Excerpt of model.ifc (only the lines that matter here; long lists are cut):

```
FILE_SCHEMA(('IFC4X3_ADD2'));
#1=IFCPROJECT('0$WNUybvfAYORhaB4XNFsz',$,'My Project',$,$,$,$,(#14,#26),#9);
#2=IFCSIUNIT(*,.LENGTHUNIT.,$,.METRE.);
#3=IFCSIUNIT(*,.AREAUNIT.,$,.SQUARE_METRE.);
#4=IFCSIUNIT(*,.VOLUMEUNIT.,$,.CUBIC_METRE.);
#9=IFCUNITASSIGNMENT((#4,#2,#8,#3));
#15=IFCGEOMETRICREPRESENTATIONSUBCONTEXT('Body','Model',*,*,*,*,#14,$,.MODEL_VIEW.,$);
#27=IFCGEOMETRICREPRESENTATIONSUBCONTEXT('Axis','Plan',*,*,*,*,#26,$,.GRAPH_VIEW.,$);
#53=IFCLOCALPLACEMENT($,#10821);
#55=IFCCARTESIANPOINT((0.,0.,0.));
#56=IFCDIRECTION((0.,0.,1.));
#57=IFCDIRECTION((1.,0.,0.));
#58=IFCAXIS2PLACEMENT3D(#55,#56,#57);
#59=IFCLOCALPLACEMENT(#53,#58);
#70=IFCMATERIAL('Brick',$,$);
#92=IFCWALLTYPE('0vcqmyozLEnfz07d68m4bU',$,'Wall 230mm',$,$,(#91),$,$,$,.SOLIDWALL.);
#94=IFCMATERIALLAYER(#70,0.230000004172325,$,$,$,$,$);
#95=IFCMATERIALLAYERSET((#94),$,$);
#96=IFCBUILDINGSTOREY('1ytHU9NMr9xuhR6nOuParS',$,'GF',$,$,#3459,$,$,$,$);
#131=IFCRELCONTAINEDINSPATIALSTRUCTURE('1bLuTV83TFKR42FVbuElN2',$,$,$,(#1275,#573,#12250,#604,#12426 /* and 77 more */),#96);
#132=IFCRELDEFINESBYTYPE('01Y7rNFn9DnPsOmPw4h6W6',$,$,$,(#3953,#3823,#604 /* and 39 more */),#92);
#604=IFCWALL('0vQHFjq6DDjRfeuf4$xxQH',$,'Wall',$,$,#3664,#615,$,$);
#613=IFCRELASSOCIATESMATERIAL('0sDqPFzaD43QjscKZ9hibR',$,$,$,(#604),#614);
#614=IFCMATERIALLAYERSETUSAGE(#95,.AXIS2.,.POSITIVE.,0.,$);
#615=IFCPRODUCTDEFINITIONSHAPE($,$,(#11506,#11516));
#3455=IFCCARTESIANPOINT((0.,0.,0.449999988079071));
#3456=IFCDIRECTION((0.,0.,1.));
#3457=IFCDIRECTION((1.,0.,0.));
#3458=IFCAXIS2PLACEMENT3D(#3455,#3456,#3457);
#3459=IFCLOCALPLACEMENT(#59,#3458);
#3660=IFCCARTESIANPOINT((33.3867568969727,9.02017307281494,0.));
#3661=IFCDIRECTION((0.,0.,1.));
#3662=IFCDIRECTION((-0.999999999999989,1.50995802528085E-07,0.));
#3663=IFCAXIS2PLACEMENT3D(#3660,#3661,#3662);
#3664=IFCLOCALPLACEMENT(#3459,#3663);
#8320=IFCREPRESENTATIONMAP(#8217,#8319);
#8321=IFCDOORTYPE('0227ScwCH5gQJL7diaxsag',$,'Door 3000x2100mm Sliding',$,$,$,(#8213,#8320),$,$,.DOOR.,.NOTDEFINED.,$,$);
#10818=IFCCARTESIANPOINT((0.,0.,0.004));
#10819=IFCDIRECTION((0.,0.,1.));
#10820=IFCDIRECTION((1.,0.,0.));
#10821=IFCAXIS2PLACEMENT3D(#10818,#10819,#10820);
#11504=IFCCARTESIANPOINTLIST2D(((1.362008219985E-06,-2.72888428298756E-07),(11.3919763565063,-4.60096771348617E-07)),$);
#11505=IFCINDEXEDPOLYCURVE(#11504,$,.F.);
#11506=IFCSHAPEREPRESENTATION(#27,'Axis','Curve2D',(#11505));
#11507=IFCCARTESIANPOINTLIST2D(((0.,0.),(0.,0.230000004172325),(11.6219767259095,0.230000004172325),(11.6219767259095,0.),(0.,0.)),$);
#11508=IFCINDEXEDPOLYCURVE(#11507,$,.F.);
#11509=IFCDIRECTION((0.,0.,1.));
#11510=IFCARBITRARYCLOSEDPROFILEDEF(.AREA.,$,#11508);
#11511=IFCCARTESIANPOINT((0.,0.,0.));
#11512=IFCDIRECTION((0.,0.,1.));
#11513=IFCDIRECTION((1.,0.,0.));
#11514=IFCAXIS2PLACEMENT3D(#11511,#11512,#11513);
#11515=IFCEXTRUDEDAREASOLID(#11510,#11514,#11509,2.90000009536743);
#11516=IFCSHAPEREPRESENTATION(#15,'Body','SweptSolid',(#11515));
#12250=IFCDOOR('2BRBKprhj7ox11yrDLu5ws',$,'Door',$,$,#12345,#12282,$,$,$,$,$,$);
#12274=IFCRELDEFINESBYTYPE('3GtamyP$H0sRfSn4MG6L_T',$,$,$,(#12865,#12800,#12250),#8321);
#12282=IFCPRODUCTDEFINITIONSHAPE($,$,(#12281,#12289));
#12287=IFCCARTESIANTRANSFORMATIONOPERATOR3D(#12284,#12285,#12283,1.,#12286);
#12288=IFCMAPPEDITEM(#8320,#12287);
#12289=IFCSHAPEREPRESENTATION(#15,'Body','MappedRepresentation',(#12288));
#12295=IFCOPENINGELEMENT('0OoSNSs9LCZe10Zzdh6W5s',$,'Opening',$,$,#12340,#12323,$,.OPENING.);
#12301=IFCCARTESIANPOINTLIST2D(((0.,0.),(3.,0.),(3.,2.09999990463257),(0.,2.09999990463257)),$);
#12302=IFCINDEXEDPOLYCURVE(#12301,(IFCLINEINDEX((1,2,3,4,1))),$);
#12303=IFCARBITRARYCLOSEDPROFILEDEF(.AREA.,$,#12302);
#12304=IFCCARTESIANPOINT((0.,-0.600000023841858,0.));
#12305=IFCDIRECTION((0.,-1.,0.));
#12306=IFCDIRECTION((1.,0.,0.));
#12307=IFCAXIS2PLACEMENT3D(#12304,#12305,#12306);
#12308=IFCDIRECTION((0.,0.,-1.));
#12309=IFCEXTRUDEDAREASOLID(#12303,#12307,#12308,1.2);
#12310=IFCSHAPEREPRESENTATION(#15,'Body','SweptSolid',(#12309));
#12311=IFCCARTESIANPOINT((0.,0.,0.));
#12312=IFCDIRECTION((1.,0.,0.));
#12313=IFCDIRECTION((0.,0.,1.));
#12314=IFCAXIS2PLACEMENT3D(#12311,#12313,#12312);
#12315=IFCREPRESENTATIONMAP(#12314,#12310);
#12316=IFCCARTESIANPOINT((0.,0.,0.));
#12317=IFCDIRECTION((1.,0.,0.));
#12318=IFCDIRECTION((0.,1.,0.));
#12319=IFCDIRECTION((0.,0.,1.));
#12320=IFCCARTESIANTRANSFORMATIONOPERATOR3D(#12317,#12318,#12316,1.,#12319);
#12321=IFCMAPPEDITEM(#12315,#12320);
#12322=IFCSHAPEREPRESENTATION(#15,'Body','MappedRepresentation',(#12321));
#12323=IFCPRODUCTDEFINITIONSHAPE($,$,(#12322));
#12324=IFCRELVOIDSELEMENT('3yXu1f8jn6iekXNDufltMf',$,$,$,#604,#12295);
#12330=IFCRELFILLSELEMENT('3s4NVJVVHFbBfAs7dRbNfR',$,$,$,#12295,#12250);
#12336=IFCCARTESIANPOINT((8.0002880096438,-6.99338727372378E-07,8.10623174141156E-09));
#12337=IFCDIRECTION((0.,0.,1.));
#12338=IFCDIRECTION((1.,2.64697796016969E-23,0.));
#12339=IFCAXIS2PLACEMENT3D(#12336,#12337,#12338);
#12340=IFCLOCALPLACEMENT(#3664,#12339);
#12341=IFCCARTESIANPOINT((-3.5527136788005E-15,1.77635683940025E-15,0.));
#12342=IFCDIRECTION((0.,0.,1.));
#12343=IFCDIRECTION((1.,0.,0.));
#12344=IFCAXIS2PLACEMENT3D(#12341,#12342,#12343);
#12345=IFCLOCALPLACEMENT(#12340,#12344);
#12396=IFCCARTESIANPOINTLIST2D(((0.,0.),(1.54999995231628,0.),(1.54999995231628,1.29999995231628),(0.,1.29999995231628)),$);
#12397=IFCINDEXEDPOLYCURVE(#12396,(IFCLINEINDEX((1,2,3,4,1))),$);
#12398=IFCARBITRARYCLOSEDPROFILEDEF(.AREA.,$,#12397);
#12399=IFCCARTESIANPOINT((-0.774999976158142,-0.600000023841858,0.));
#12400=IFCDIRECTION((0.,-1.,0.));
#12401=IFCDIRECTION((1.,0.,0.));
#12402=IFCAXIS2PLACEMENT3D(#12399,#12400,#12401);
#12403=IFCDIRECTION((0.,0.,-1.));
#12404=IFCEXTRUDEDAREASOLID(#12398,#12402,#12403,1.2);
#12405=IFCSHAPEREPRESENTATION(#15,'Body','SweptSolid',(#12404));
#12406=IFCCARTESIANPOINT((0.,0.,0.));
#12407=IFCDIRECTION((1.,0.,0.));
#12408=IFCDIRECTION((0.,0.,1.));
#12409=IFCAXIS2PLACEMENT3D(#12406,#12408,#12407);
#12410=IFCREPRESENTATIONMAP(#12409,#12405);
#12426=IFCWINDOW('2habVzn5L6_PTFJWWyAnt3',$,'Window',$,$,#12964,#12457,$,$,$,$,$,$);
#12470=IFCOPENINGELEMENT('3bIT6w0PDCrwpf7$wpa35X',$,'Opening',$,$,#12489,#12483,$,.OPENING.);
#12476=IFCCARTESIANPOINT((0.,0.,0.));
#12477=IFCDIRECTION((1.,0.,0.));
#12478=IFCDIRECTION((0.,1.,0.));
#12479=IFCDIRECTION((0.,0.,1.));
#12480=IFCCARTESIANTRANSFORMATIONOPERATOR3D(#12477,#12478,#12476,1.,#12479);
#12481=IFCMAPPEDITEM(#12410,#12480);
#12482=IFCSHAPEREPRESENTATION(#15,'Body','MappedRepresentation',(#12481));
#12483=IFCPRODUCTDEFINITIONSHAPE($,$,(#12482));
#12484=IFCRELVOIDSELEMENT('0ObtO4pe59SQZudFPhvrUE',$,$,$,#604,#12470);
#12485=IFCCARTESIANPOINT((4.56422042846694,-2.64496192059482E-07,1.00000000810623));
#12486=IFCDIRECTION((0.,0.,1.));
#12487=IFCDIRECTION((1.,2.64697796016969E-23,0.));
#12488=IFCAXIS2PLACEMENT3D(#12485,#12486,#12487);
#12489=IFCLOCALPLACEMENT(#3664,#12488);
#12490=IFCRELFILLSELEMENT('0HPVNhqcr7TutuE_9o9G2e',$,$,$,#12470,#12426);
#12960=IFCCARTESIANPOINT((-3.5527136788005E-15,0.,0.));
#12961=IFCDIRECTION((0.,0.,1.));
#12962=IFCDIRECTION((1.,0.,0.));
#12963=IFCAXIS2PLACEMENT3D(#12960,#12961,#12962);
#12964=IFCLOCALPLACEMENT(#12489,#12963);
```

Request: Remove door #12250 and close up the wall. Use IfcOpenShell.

```python
import ifcopenshell
import ifcopenshell.api.feature
import ifcopenshell.api.root
import ifcopenshell.geom
import ifcopenshell.util.shape

model = ifcopenshell.open("model.ifc")
settings = ifcopenshell.geom.settings()


def volume(element):
    """Net volume in cubic metres, openings subtracted."""
    shape = ifcopenshell.geom.create_shape(settings, element)
    return ifcopenshell.util.shape.get_volume(shape.geometry)


door = model.by_guid("2BRBKprhj7ox11yrDLu5ws")
opening = door.FillsVoids[0].RelatingOpeningElement
wall = opening.VoidsElements[0].RelatingBuildingElement
before = volume(wall)

ifcopenshell.api.root.remove_product(model, product=door)
ifcopenshell.api.feature.remove_feature(model, feature=opening)

after = volume(wall)

print(f"wall volume {before:.3f} -> {after:.3f} m3")

model.write("model_updated.ifc")
```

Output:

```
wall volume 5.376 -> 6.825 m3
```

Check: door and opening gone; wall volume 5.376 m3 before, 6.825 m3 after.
